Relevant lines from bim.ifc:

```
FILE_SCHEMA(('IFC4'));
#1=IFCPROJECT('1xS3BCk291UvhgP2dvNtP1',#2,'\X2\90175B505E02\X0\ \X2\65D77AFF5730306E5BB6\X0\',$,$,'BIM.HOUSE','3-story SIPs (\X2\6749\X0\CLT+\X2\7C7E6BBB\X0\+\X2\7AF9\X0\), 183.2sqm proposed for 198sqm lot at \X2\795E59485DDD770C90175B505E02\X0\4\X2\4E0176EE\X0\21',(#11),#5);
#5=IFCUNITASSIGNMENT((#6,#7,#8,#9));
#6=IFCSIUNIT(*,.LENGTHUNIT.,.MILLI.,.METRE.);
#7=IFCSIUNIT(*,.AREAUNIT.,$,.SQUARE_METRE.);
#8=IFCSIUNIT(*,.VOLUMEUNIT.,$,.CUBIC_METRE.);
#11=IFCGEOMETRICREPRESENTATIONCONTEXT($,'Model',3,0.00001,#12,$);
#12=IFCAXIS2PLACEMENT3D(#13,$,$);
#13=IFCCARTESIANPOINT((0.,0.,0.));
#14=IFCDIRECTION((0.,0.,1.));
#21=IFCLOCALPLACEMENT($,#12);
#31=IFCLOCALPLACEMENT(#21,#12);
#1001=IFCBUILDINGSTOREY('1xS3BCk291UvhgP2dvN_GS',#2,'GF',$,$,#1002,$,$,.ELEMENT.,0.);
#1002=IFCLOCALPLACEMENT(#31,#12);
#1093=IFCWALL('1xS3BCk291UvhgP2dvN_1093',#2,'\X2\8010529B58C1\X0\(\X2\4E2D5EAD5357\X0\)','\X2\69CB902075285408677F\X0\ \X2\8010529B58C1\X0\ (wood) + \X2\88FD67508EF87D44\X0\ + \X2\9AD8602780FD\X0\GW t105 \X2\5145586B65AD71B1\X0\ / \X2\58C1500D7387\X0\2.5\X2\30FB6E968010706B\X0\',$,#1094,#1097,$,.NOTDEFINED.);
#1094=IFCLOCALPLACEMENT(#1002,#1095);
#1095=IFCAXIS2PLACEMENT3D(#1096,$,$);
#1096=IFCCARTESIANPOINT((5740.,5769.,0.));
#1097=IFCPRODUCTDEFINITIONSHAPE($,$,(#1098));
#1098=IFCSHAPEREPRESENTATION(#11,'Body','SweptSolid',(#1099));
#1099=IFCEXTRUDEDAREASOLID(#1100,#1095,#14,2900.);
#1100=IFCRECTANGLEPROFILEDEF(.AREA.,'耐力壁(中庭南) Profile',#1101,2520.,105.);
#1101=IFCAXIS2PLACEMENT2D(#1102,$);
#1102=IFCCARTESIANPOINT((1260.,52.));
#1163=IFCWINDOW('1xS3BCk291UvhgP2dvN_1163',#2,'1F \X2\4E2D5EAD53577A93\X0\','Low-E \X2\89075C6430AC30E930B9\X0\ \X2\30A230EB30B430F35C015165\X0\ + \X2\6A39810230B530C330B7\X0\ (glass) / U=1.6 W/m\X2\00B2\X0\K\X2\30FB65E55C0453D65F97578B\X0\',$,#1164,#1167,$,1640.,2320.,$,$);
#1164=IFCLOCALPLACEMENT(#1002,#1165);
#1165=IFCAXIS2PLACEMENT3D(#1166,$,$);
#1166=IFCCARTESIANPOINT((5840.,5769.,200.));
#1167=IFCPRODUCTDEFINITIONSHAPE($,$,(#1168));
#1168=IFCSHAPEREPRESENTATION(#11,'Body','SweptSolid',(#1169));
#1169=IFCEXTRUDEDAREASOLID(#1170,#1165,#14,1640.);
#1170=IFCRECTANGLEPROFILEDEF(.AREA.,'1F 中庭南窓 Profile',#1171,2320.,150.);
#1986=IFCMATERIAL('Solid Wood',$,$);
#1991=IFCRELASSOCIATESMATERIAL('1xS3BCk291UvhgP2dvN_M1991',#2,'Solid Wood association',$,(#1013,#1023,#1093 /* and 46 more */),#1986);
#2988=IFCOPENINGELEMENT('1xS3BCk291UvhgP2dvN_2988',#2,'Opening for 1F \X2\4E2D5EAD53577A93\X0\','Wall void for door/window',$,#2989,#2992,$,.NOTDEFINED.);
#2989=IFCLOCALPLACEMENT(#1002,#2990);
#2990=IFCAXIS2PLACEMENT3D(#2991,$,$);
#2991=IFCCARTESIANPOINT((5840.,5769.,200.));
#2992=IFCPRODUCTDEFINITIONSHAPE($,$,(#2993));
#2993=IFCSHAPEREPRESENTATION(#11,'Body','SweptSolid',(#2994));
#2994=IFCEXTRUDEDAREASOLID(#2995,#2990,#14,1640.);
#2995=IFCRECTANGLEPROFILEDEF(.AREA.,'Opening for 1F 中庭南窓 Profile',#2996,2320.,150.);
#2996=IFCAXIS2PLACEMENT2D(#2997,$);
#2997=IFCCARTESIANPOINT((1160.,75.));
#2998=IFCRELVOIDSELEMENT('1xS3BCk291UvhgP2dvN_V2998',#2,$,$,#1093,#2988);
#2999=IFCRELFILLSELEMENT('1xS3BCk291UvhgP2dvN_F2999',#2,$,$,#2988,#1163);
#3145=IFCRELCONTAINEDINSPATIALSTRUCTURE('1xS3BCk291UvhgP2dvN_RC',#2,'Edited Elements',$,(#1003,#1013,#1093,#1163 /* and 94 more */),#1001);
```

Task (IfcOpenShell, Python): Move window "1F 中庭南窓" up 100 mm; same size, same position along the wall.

```python
import numpy as np
import ifcopenshell
import ifcopenshell.api.geometry
import ifcopenshell.util.placement
import ifcopenshell.util.unit

model = ifcopenshell.open("bim.ifc")
unit_scale = ifcopenshell.util.unit.calculate_unit_scale(model)

window = model.by_guid("1xS3BCk291UvhgP2dvN_1163")
opening = window.FillsVoids[0].RelatingOpeningElement
dz = 0.1 / unit_scale

shift = np.array([0.0, 0.0, dz])
# The window is not placed relative to its opening, so move both.
for product in (opening, window):
    matrix = ifcopenshell.util.placement.get_local_placement(product.ObjectPlacement)
    matrix[:3, 3] += shift
    ifcopenshell.api.geometry.edit_object_placement(model, product=product, matrix=matrix, is_si=False)

print(f"moved by {dz * unit_scale:+.3f} m")

model.write("bim_rev.ifc")
```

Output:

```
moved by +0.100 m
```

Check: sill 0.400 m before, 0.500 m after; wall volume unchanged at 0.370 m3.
